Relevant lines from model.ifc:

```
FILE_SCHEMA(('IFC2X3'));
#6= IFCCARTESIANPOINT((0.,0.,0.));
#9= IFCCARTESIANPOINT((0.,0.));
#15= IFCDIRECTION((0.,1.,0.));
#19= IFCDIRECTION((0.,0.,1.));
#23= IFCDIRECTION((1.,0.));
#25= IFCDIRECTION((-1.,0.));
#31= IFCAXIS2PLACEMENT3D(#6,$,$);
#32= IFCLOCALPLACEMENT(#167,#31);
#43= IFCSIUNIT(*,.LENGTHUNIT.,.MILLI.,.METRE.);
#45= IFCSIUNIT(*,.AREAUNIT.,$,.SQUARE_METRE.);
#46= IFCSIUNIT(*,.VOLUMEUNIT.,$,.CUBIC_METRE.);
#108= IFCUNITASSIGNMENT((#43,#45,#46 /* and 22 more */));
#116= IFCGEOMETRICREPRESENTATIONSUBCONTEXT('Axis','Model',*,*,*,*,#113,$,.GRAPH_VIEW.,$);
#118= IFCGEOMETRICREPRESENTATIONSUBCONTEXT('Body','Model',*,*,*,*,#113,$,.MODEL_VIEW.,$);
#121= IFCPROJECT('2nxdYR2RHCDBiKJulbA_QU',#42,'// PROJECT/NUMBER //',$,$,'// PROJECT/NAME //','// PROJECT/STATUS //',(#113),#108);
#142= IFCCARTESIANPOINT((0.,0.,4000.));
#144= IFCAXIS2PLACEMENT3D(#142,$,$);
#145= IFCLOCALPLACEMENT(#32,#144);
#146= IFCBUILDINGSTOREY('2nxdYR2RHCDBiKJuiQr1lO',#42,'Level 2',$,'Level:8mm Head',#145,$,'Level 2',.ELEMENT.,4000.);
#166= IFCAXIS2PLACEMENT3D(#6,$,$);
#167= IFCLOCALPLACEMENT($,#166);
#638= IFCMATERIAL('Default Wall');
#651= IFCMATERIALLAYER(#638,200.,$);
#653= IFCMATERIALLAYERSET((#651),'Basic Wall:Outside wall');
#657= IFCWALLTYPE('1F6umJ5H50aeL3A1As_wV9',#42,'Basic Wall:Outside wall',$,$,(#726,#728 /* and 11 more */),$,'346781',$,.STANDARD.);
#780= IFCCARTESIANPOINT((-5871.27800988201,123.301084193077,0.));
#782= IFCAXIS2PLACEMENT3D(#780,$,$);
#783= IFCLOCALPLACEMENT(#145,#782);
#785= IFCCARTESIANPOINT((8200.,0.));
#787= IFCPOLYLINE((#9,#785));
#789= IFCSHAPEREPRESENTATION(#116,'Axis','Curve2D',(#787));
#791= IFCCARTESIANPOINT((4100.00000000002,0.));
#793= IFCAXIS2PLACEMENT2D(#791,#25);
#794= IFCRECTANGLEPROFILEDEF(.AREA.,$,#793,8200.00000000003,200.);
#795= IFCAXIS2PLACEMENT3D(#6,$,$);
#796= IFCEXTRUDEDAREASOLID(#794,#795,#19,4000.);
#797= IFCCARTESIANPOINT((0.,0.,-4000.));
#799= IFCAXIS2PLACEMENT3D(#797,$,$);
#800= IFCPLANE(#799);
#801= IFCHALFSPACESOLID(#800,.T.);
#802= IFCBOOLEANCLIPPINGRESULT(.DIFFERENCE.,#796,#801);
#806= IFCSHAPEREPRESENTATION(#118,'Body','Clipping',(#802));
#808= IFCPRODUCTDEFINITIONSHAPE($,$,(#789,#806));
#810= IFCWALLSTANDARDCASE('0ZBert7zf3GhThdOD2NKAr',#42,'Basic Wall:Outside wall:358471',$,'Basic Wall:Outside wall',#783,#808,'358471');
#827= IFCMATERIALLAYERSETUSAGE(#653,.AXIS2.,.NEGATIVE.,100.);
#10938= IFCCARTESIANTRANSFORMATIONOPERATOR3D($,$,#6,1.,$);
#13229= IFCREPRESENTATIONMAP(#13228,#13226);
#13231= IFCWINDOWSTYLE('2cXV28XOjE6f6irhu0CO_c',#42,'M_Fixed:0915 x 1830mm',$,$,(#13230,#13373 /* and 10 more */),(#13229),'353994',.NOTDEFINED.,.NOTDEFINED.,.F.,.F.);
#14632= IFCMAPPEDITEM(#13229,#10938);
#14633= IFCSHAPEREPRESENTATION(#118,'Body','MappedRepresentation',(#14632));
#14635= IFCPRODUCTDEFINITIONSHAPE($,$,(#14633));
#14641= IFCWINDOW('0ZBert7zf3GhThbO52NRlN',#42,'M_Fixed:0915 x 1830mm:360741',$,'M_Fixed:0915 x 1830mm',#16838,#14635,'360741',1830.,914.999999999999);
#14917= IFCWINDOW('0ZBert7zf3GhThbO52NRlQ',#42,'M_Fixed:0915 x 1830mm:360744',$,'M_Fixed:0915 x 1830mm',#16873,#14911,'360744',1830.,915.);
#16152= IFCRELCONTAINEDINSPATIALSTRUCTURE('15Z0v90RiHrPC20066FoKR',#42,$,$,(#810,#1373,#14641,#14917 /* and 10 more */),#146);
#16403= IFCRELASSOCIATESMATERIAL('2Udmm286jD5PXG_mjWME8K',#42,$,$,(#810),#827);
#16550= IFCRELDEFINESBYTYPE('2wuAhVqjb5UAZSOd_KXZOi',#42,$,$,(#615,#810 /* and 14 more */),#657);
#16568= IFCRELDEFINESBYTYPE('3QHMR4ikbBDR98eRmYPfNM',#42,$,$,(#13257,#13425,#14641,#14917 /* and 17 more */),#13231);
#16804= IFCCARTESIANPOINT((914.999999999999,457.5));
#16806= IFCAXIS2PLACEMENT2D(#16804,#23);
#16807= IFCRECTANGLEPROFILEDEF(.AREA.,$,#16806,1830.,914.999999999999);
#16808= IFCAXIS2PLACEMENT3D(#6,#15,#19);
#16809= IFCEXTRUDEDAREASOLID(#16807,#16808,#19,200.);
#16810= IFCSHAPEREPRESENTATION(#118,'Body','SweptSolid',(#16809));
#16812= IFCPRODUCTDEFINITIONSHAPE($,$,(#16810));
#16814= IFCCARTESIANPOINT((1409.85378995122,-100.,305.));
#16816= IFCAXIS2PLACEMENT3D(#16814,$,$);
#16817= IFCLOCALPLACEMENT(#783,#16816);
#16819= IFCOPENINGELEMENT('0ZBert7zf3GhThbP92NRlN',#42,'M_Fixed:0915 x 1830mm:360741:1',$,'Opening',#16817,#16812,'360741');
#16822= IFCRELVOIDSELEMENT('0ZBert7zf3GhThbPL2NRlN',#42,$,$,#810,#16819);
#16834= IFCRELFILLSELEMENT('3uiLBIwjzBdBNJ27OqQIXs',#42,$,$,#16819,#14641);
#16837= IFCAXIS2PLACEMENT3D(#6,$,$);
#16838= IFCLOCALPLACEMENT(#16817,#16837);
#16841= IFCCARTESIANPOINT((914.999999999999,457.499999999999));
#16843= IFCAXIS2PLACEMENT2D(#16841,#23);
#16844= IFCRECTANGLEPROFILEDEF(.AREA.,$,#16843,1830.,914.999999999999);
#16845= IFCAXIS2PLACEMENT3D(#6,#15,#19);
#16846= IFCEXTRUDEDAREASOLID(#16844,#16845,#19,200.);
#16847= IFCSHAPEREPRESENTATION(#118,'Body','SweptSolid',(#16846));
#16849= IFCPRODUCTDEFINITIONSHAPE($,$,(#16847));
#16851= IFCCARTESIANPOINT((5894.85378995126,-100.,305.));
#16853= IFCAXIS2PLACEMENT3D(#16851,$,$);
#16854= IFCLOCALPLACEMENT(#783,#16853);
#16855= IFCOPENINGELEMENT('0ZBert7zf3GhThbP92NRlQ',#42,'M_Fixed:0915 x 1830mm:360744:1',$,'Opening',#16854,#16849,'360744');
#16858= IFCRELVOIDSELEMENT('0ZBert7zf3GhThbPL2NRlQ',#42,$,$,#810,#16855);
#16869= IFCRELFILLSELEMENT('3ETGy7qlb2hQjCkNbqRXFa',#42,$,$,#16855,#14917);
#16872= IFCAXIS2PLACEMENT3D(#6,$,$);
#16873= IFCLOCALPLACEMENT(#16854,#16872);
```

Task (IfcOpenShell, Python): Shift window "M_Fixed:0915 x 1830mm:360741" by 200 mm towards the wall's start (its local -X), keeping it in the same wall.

```python
import ifcopenshell
import ifcopenshell.api.geometry
import ifcopenshell.util.placement
import ifcopenshell.util.unit

model = ifcopenshell.open("model.ifc")
unit_scale = ifcopenshell.util.unit.calculate_unit_scale(model)

window = model.by_guid("0ZBert7zf3GhThbO52NRlN")
opening = window.FillsVoids[0].RelatingOpeningElement
wall = opening.VoidsElements[0].RelatingBuildingElement

wall_matrix = ifcopenshell.util.placement.get_local_placement(wall.ObjectPlacement)
shift = wall_matrix[:3, 0] * -0.2 / unit_scale
before = ifcopenshell.util.placement.get_local_placement(window.ObjectPlacement)[:3, 3].copy()

# The window is placed relative to its opening, so it follows when the opening moves.
matrix = ifcopenshell.util.placement.get_local_placement(opening.ObjectPlacement)
matrix[:3, 3] += shift
ifcopenshell.api.geometry.edit_object_placement(
    model, product=opening, matrix=matrix, is_si=False, should_transform_children=True
)

after = ifcopenshell.util.placement.get_local_placement(window.ObjectPlacement)[:3, 3]
print("window moved by", (after - before).round(3) + 0.0)

model.write("model-out.ifc")
```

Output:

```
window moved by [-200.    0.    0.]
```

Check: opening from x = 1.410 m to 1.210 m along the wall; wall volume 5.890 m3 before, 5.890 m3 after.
